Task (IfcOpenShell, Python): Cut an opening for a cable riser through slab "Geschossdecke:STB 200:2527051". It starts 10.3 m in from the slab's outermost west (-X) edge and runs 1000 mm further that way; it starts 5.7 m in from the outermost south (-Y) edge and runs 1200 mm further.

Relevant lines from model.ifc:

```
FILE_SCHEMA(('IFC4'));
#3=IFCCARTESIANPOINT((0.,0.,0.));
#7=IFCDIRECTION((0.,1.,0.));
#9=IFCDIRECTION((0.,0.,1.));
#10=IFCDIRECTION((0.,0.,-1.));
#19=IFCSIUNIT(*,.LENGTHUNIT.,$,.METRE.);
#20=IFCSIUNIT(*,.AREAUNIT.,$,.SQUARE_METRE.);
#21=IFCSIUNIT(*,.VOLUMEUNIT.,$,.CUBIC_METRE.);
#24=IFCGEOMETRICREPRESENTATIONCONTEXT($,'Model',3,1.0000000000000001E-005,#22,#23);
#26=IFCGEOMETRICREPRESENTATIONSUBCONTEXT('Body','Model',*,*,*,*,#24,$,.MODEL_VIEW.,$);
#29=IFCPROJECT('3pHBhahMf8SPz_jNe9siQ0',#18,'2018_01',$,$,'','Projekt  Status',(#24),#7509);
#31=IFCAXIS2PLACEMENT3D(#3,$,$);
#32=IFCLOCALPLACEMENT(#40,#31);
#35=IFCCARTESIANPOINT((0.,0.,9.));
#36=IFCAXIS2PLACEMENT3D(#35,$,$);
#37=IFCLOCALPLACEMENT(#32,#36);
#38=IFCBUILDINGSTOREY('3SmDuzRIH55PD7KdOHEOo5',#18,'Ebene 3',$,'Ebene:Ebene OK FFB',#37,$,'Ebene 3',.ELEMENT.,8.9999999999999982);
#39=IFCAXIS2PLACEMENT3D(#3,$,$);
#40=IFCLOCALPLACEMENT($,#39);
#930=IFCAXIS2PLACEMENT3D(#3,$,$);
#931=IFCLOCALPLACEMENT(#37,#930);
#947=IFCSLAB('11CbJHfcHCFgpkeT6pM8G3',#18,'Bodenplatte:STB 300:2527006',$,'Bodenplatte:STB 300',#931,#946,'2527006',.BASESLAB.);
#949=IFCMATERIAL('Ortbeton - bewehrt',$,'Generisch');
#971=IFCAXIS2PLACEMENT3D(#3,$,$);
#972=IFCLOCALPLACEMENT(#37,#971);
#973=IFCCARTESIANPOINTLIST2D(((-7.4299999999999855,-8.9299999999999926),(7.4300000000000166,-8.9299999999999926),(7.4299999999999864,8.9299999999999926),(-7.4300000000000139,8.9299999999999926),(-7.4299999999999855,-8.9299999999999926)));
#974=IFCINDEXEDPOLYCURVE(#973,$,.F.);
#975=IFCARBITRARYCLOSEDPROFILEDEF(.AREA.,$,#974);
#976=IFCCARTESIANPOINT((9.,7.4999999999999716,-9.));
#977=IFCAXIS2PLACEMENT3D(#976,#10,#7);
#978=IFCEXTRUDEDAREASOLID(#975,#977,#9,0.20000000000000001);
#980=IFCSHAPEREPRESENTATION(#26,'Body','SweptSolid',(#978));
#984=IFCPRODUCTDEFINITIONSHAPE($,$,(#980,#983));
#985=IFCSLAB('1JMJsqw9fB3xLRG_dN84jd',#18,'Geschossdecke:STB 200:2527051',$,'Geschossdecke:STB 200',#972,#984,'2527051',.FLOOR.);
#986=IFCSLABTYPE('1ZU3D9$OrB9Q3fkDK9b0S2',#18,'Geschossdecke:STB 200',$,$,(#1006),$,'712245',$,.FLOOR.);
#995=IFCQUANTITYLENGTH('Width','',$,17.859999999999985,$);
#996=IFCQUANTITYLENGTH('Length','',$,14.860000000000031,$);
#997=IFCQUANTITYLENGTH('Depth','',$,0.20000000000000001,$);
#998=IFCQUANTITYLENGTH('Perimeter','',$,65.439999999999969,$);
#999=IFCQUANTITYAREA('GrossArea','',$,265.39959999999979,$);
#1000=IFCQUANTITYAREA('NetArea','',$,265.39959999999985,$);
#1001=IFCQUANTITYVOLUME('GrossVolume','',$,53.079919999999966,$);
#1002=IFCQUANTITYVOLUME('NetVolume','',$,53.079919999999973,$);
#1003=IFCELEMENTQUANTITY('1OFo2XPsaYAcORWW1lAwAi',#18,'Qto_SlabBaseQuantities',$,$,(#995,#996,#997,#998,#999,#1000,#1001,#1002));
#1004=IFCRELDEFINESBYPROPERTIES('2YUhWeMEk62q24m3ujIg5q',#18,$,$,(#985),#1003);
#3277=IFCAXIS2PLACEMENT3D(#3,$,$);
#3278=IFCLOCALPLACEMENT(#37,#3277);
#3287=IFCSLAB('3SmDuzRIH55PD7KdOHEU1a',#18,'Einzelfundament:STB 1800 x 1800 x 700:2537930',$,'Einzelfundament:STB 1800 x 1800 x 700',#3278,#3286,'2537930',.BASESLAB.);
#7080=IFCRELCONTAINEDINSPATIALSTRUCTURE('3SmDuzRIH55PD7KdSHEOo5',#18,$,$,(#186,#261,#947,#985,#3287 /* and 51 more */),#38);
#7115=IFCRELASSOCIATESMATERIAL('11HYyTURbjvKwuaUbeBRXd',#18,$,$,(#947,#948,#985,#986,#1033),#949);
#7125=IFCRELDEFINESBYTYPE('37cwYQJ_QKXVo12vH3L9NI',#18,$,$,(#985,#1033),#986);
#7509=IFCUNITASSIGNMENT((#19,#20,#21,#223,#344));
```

```python
import numpy as np
import ifcopenshell
import ifcopenshell.api.feature
import ifcopenshell.api.geometry
import ifcopenshell.api.pset
import ifcopenshell.api.root
import ifcopenshell.geom
import ifcopenshell.util.element
import ifcopenshell.util.placement
import ifcopenshell.util.representation
import ifcopenshell.util.shape
import ifcopenshell.util.unit

model = ifcopenshell.open("model.ifc")
unit_scale = ifcopenshell.util.unit.calculate_unit_scale(model)
area_scale = ifcopenshell.util.unit.calculate_unit_scale(model, "AREAUNIT")
volume_scale = ifcopenshell.util.unit.calculate_unit_scale(model, "VOLUMEUNIT")
settings = ifcopenshell.geom.settings()


def volume(element):
    """Net volume in cubic metres, openings subtracted."""
    shape = ifcopenshell.geom.create_shape(settings, element)
    return ifcopenshell.util.shape.get_volume(shape.geometry)


slab = model.by_guid("1JMJsqw9fB3xLRG_dN84jd")
before = volume(slab)

# Extent in the slab's own axes, in metres. The edges named are its -X and -Y sides.
slab_shape = ifcopenshell.geom.create_shape(settings, slab)
vertices = ifcopenshell.util.shape.get_vertices(slab_shape.geometry)
x_min, y_min, bottom = vertices.min(axis=0)
top = vertices[:, 2].max()

opening = ifcopenshell.api.root.create_entity(model, ifc_class="IfcOpeningElement", name="Cable riser opening", predefined_type="OPENING")
context = ifcopenshell.util.representation.get_context(model, "Model", "Body", "MODEL_VIEW")
width, depth = 1, 1.2
outline = [(0.0, 0.0), (width, 0.0), (width, depth), (0.0, depth), (0.0, 0.0)]
# Overshoot both faces by 50 mm so the cut is clean.
shape = ifcopenshell.api.geometry.add_slab_representation(
    model, context=context, depth=top - bottom + 0.1, polyline=outline
)
ifcopenshell.api.geometry.assign_representation(model, product=opening, representation=shape)

matrix = ifcopenshell.util.placement.get_local_placement(slab.ObjectPlacement)
matrix[:, 3] = matrix @ np.append(np.array([x_min + 10.3, y_min + 5.7, bottom - 0.05]) / unit_scale, 1.0)
ifcopenshell.api.geometry.edit_object_placement(model, product=opening, matrix=matrix, is_si=False)
ifcopenshell.api.feature.add_feature(model, feature=opening, element=slab)

after = volume(slab)

# Update the slab's stored quantities.
qto = model.by_id(ifcopenshell.util.element.get_pset(slab, "Qto_SlabBaseQuantities", should_inherit=False)["id"])
ifcopenshell.api.pset.edit_qto(model, qto=qto, properties={
    "NetArea": after / (top - bottom) / area_scale,
    "NetVolume": after / volume_scale,
})

print(f"slab volume {before:.3f} -> {after:.3f} m3")

model.write("model_edited.ifc")
```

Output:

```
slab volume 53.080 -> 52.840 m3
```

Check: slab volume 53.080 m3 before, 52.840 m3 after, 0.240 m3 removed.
